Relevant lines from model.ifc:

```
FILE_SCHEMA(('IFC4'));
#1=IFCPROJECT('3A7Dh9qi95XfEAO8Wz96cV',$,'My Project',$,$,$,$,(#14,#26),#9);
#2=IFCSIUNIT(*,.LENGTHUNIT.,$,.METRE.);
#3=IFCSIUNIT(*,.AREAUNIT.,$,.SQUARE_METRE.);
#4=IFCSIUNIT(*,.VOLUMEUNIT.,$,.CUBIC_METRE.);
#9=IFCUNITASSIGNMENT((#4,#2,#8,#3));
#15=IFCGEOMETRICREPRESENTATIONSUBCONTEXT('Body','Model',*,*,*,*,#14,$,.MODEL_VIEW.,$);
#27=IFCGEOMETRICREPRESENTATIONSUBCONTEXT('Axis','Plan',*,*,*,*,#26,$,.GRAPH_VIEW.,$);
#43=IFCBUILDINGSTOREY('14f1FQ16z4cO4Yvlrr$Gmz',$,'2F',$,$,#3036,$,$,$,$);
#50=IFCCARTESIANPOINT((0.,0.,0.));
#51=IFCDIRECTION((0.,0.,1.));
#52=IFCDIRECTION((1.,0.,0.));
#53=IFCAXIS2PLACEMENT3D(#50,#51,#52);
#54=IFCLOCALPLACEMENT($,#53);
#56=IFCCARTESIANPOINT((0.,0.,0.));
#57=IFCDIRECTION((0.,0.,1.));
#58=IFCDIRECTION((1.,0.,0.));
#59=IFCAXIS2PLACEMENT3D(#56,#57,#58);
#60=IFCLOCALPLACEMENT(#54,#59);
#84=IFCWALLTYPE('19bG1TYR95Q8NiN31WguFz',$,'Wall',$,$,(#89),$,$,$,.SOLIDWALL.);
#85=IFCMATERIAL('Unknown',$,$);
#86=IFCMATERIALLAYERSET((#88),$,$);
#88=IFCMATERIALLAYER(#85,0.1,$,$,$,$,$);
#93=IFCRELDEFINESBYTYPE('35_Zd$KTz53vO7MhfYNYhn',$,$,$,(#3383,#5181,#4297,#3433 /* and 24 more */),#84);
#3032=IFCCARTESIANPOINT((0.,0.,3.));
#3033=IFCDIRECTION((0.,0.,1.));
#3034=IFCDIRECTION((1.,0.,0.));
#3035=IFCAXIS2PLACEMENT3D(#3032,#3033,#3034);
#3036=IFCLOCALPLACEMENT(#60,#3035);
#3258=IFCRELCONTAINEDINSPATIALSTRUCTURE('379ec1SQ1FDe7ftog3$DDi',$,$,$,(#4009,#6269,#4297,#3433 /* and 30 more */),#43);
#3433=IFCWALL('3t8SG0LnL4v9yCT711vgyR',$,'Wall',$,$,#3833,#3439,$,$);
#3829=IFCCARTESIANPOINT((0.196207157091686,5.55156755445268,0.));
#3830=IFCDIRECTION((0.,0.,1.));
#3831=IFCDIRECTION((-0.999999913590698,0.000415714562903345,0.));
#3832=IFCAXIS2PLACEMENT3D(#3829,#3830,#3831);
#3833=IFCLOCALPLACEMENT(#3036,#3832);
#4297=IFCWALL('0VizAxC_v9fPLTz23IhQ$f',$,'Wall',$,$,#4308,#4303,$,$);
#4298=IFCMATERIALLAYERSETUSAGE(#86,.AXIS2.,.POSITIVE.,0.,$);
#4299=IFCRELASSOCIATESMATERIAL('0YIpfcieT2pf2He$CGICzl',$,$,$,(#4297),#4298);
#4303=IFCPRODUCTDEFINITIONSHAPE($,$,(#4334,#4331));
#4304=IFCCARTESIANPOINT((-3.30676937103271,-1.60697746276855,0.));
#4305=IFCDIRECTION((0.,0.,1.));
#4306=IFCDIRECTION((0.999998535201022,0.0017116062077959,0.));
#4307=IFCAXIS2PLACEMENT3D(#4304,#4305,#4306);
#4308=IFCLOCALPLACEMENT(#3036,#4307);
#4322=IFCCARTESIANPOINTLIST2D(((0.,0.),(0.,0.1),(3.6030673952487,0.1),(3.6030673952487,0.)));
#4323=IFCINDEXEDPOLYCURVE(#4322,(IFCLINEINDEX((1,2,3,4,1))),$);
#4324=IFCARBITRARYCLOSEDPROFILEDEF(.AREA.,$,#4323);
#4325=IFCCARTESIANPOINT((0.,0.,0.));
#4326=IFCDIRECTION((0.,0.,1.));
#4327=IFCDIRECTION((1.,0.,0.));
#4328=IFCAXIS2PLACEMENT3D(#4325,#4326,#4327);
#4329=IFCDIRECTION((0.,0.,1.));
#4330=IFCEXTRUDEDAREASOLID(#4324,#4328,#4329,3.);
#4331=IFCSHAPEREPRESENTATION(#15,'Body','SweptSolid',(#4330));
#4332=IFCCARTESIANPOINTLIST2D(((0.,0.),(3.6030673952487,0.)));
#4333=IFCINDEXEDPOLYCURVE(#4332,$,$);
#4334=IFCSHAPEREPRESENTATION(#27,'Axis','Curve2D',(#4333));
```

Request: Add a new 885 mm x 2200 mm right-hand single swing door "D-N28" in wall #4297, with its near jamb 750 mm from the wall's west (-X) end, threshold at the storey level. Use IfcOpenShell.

```python
import numpy as np
import ifcopenshell
import ifcopenshell.api.feature
import ifcopenshell.api.geometry
import ifcopenshell.api.root
import ifcopenshell.api.spatial
import ifcopenshell.geom
import ifcopenshell.util.element
import ifcopenshell.util.placement
import ifcopenshell.util.representation
import ifcopenshell.util.shape
import ifcopenshell.util.unit

model = ifcopenshell.open("model.ifc")
unit_scale = ifcopenshell.util.unit.calculate_unit_scale(model)
settings = ifcopenshell.geom.settings()


def volume(element):
    """Net volume in cubic metres, openings subtracted."""
    shape = ifcopenshell.geom.create_shape(settings, element)
    return ifcopenshell.util.shape.get_volume(shape.geometry)


wall = model.by_id(4297)
storey = ifcopenshell.util.element.get_container(wall, ifc_class="IfcBuildingStorey")
context = ifcopenshell.util.representation.get_context(model, "Model", "Body", "MODEL_VIEW")
before = volume(wall)

width, height, from_end, sill = 0.885, 2.2, 0.75, 0.0  # metres

# The wall runs along its own X axis, and the end named is its -X end.
wall_shape = ifcopenshell.geom.create_shape(settings, wall)
x, y, z = ifcopenshell.util.shape.get_vertices(wall_shape.geometry).T
start = x.min() + from_end
face, thickness = float(y.min()), float(y.max() - y.min())
wall_matrix = ifcopenshell.util.placement.get_local_placement(wall.ObjectPlacement)
level = ifcopenshell.util.placement.get_local_placement(storey.ObjectPlacement)[2, 3]


def in_wall(x, y):
    """Placement at x, y metres in the wall's axes, at sill height."""
    matrix = wall_matrix.copy()
    matrix[:, 3] = wall_matrix @ np.array([x / unit_scale, y / unit_scale, 0.0, 1.0])
    matrix[2, 3] = level + sill / unit_scale
    return matrix


# Opening: a box that overshoots both wall faces by 50 mm.
opening = ifcopenshell.api.root.create_entity(model, ifc_class="IfcOpeningElement", predefined_type="OPENING")
box = ifcopenshell.api.geometry.add_wall_representation(
    model, context=context, length=width, height=height, thickness=thickness + 0.1
)
ifcopenshell.api.geometry.assign_representation(model, product=opening, representation=box)
ifcopenshell.api.geometry.edit_object_placement(model, product=opening, matrix=in_wall(start, face - 0.05), is_si=False)
ifcopenshell.api.feature.add_feature(model, feature=opening, element=wall)

door = ifcopenshell.api.root.create_entity(model, ifc_class="IfcDoor", name="D-N28", predefined_type="DOOR")
door.OverallWidth, door.OverallHeight = width / unit_scale, height / unit_scale
door.OperationType = "SINGLE_SWING_RIGHT"
body = ifcopenshell.api.geometry.add_door_representation(
    model,
    context=context,
    overall_width=door.OverallWidth,
    overall_height=door.OverallHeight,
    operation_type="SINGLE_SWING_RIGHT",
    lining_properties={"LiningDepth": thickness / unit_scale, "ThresholdDepth": thickness / unit_scale},
)
ifcopenshell.api.geometry.assign_representation(model, product=door, representation=body)
ifcopenshell.api.spatial.assign_container(model, products=[door], relating_structure=storey)
ifcopenshell.api.feature.add_filling(model, opening=opening, element=door)

# The lining spans the wall, so the door starts at the wall face.
ifcopenshell.api.geometry.edit_object_placement(model, product=door, matrix=in_wall(start, face), is_si=False)

after = volume(wall)

print(f"wall volume {before:.3f} -> {after:.3f} m3")

model.write("model_v2.ifc")
```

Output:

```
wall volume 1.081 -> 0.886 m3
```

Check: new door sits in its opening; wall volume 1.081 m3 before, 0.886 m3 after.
